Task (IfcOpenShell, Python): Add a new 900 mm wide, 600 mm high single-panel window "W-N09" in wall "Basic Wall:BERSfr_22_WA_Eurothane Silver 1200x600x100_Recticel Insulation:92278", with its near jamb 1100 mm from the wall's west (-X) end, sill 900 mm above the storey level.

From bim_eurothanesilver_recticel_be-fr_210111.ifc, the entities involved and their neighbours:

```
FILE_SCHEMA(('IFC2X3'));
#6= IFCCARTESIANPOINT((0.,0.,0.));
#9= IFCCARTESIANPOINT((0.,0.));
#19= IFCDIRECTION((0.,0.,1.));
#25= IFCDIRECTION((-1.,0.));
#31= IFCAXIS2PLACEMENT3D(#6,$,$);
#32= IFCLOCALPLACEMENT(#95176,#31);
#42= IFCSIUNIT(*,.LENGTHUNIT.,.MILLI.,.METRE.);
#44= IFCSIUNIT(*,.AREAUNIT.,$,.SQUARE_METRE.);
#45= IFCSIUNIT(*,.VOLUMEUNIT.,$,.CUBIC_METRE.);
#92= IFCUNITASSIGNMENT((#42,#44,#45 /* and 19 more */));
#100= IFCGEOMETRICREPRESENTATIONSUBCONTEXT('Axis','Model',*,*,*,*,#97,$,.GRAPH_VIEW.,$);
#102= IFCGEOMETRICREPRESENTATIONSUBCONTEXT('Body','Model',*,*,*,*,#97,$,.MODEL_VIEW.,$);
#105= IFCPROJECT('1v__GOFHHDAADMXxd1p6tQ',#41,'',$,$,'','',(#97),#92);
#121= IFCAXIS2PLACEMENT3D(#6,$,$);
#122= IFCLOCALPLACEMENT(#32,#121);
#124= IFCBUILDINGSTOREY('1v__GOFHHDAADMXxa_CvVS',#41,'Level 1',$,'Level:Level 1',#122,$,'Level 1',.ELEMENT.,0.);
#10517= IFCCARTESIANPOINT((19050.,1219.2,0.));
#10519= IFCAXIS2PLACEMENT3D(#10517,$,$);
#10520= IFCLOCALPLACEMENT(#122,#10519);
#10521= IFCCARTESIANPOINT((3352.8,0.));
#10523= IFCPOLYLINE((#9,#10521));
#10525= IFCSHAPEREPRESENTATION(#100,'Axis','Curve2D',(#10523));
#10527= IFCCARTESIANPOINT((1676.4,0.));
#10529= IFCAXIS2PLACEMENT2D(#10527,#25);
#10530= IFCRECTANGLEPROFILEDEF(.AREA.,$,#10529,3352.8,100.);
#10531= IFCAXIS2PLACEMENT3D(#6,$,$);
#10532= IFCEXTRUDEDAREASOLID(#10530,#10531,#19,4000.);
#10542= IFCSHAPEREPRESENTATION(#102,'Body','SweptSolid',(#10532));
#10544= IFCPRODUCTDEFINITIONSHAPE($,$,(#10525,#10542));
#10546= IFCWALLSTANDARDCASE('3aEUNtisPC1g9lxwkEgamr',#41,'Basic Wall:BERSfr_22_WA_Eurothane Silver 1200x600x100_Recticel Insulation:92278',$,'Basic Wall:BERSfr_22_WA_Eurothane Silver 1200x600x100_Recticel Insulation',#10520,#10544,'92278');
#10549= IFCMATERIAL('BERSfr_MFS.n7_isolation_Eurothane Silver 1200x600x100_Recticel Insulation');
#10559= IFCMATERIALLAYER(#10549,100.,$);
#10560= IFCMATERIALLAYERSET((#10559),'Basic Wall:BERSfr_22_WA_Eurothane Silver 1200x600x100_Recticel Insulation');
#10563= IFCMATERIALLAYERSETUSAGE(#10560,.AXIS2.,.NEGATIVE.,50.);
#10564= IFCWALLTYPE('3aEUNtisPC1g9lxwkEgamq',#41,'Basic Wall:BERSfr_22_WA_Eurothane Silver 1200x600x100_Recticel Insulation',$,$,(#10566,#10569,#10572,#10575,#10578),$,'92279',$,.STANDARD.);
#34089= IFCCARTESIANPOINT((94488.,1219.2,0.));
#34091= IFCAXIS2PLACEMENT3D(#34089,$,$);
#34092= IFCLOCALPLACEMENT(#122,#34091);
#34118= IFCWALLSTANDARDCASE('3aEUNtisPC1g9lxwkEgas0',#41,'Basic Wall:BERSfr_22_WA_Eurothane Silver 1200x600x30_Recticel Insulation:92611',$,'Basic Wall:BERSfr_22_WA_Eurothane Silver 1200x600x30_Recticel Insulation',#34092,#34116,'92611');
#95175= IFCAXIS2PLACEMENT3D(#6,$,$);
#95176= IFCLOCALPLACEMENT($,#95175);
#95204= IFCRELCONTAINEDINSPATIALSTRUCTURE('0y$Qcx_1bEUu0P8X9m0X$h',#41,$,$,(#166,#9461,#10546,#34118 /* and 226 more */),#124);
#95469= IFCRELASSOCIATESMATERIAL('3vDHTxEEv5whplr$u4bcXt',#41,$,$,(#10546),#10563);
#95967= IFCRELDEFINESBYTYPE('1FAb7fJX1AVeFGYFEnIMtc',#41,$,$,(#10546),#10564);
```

```python
import numpy as np
import ifcopenshell
import ifcopenshell.api.feature
import ifcopenshell.api.geometry
import ifcopenshell.api.root
import ifcopenshell.api.spatial
import ifcopenshell.api.type
import ifcopenshell.geom
import ifcopenshell.util.element
import ifcopenshell.util.placement
import ifcopenshell.util.representation
import ifcopenshell.util.shape
import ifcopenshell.util.unit

model = ifcopenshell.open("bim_eurothanesilver_recticel_be-fr_210111.ifc")
unit_scale = ifcopenshell.util.unit.calculate_unit_scale(model)
settings = ifcopenshell.geom.settings()


def volume(element):
    """Net volume in cubic metres, openings subtracted."""
    shape = ifcopenshell.geom.create_shape(settings, element)
    return ifcopenshell.util.shape.get_volume(shape.geometry)


wall = model.by_guid("3aEUNtisPC1g9lxwkEgamr")
storey = ifcopenshell.util.element.get_container(wall, ifc_class="IfcBuildingStorey")
context = ifcopenshell.util.representation.get_context(model, "Model", "Body", "MODEL_VIEW")
before = volume(wall)

width, height, from_end, sill = 0.9, 0.6, 1.1, 0.9  # metres

# The wall runs along its own X axis, and the end named is its -X end.
wall_shape = ifcopenshell.geom.create_shape(settings, wall)
x, y, z = ifcopenshell.util.shape.get_vertices(wall_shape.geometry).T
start = x.min() + from_end
face, thickness = float(y.min()), float(y.max() - y.min())
wall_matrix = ifcopenshell.util.placement.get_local_placement(wall.ObjectPlacement)
level = ifcopenshell.util.placement.get_local_placement(storey.ObjectPlacement)[2, 3]


def in_wall(x, y):
    """Placement at x, y metres in the wall's axes, at sill height."""
    matrix = wall_matrix.copy()
    matrix[:, 3] = wall_matrix @ np.array([x / unit_scale, y / unit_scale, 0.0, 1.0])
    matrix[2, 3] = level + sill / unit_scale
    return matrix


# Opening: a box that overshoots both wall faces by 50 mm.
opening = ifcopenshell.api.root.create_entity(model, ifc_class="IfcOpeningElement")
box = ifcopenshell.api.geometry.add_wall_representation(
    model, context=context, length=width, height=height, thickness=thickness + 0.1
)
ifcopenshell.api.geometry.assign_representation(model, product=opening, representation=box)
ifcopenshell.api.geometry.edit_object_placement(model, product=opening, matrix=in_wall(start, face - 0.05), is_si=False)
ifcopenshell.api.feature.add_feature(model, feature=opening, element=wall)

window = ifcopenshell.api.root.create_entity(model, ifc_class="IfcWindow", name="W-N09")
window.OverallWidth, window.OverallHeight = width / unit_scale, height / unit_scale
body = ifcopenshell.api.geometry.add_window_representation(
    model,
    context=context,
    overall_width=window.OverallWidth,
    overall_height=window.OverallHeight,
    partition_type="SINGLE_PANEL",
)
ifcopenshell.api.geometry.assign_representation(model, product=window, representation=body)
ifcopenshell.api.spatial.assign_container(model, products=[window], relating_structure=storey)
fills = ifcopenshell.api.feature.add_filling(model, opening=opening, element=window)
fills.OwnerHistory = window.OwnerHistory  # required in IFC2X3

# IFC2X3 keeps the operation on the window style.
style = ifcopenshell.api.root.create_entity(model, ifc_class="IfcWindowStyle", name="W-N09")
style.OperationType, style.ConstructionType = "SINGLE_PANEL", "NOTDEFINED"
style.ParameterTakesPrecedence = style.Sizeable = False
ifcopenshell.api.type.assign_type(model, related_objects=[window], relating_type=style)

# Centre the window in the wall's thickness.
ifcopenshell.api.geometry.edit_object_placement(model, product=window, matrix=in_wall(start, face), is_si=False)
window_shape = ifcopenshell.geom.create_shape(settings, window)
depth = ifcopenshell.util.shape.get_vertices(window_shape.geometry)[:, 1]
offset = face + thickness / 2 - (depth.min() + depth.max()) / 2
ifcopenshell.api.geometry.edit_object_placement(model, product=window, matrix=in_wall(start, offset), is_si=False)

after = volume(wall)

print(f"wall volume {before:.3f} -> {after:.3f} m3")

model.write("bim_eurothanesilver_recticel_be-fr_210111_v2.ifc")
```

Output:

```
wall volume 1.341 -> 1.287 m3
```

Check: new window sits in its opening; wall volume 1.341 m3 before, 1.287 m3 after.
